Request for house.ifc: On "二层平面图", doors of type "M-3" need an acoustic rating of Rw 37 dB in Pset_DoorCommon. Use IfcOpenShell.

First a look at what the model holds.

```python
import ifcopenshell
import ifcopenshell.util.element

model = ifcopenshell.open("house.ifc")
print(model.schema)
storey = next(s for s in model.by_type("IfcBuildingStorey") if s.Name == "二层平面图")
doors = [e for e in ifcopenshell.util.element.get_decomposition(storey) if e.is_a("IfcDoor")]
seen = {}
for e in doors:
    element_type = ifcopenshell.util.element.get_type(e)
    key = (element_type.Name if element_type != e and element_type else None, ifcopenshell.util.element.get_pset(e, "Pset_DoorCommon", "AcousticRating"))
    seen[key] = seen.get(key, 0) + 1
for (name, value), count in sorted(seen.items(), key=str):
    print(count, "x", name, "|", value)
```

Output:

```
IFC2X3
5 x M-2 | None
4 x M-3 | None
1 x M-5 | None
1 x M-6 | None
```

```python
import ifcopenshell
import ifcopenshell.api.pset
import ifcopenshell.util.element

model = ifcopenshell.open("house.ifc")

storey = next(s for s in model.by_type("IfcBuildingStorey") if s.Name == "二层平面图")
doors = [e for e in ifcopenshell.util.element.get_decomposition(storey) if e.is_a("IfcDoor")]

count = 0
for e in doors:
    element_type = ifcopenshell.util.element.get_type(e)
    if element_type in (None, e) or element_type.Name != "M-3":
        continue
    # add_pset returns the element's existing set when there is one.
    pset = ifcopenshell.api.pset.add_pset(model, product=e, name="Pset_DoorCommon")
    ifcopenshell.api.pset.edit_pset(model, pset=pset, properties={"AcousticRating": "Rw 37 dB"})
    count += 1

print(count, "doors updated")

model.write("house-out.ifc")
```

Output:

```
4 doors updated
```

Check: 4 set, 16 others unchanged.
